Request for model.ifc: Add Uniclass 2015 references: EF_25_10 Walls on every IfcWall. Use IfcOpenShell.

First a look at what the model holds.

```python
import ifcopenshell

model = ifcopenshell.open("model.ifc")
print(model.schema)
print("classifications:", [c.Name for c in model.by_type("IfcClassification")])
for ifc_class in ("IfcDoor", "IfcRoof", "IfcStair", "IfcWall", "IfcWindow"):
    print(ifc_class, len(model.by_type(ifc_class)))
```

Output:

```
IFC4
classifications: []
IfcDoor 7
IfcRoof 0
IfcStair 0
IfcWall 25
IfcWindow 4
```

```python
import ifcopenshell
import ifcopenshell.api.classification

model = ifcopenshell.open("model.ifc")

system = ifcopenshell.api.classification.add_classification(model, classification="Uniclass 2015")

codes = {
    "IfcWall": ("EF_25_10", "Walls"),
}
for ifc_class, (code, name) in codes.items():
    products = model.by_type(ifc_class)
    ifcopenshell.api.classification.add_reference(
        model, products=products, classification=system, identification=code, name=name
    )
    print(code, len(products))

model.write("model_v2.ifc")
```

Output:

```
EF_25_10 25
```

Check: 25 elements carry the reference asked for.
